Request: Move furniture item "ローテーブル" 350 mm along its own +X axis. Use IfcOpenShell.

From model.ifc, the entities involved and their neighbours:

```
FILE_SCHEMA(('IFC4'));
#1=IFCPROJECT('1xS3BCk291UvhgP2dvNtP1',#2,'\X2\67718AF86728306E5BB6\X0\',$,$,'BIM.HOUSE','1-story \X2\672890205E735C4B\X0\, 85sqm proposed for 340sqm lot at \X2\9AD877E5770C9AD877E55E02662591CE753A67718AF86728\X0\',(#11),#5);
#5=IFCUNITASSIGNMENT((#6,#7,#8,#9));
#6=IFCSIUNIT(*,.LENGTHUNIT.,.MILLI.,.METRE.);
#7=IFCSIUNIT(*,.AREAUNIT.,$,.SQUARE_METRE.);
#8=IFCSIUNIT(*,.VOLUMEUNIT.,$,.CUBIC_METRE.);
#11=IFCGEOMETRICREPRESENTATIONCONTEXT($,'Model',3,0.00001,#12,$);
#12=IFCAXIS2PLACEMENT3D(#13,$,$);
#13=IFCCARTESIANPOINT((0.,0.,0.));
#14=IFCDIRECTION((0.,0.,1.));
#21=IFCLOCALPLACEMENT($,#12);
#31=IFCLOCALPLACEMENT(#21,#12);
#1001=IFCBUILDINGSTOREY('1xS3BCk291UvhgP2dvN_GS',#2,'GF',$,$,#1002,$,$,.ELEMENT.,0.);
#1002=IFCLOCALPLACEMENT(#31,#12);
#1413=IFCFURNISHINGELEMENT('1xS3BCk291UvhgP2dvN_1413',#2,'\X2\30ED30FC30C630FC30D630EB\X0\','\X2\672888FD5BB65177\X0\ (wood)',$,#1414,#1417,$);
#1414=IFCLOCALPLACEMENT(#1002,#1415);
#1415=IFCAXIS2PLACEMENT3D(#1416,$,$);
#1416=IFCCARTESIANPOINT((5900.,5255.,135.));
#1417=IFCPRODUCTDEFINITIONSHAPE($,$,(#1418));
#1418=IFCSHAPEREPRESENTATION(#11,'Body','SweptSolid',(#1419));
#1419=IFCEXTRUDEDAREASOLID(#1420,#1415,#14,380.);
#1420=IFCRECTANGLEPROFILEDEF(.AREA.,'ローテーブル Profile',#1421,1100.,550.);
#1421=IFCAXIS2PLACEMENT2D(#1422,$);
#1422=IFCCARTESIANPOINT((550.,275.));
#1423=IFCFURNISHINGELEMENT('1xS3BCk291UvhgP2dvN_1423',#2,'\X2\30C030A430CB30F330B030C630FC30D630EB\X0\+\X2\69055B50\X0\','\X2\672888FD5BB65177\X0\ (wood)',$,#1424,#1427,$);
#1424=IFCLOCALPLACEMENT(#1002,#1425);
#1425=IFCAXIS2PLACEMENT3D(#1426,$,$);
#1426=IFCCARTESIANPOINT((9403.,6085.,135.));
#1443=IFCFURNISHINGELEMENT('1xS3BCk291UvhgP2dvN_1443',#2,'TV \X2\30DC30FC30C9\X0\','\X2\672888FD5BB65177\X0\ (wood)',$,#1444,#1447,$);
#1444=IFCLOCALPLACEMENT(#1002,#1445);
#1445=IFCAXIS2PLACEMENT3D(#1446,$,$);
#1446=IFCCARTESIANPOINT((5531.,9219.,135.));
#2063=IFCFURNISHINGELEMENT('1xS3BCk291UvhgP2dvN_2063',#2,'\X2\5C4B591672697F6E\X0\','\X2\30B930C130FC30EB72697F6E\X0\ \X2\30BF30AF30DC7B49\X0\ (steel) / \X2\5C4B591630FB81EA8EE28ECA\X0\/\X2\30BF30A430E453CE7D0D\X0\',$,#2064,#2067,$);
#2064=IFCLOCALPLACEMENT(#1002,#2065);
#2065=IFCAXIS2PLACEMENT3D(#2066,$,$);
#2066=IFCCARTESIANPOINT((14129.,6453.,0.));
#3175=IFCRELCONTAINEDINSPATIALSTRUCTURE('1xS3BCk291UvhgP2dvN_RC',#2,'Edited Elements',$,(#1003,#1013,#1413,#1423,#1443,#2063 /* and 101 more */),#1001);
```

```python
import ifcopenshell
import ifcopenshell.api.geometry
import ifcopenshell.util.placement

model = ifcopenshell.open("model.ifc")

item = model.by_guid("1xS3BCk291UvhgP2dvN_1413")
matrix = ifcopenshell.util.placement.get_local_placement(item.ObjectPlacement)
matrix[:3, 3] += matrix[:3, 0] * 350.0
ifcopenshell.api.geometry.edit_object_placement(model, product=item, matrix=matrix, is_si=False)

print(ifcopenshell.util.placement.get_local_placement(item.ObjectPlacement).round(3) + 0.0)

model.write("model_updated.ifc")
```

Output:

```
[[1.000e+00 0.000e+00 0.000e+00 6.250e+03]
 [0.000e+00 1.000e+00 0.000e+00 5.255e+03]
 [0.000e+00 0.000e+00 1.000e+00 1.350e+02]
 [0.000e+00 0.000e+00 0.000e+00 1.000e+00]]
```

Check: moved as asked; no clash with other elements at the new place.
